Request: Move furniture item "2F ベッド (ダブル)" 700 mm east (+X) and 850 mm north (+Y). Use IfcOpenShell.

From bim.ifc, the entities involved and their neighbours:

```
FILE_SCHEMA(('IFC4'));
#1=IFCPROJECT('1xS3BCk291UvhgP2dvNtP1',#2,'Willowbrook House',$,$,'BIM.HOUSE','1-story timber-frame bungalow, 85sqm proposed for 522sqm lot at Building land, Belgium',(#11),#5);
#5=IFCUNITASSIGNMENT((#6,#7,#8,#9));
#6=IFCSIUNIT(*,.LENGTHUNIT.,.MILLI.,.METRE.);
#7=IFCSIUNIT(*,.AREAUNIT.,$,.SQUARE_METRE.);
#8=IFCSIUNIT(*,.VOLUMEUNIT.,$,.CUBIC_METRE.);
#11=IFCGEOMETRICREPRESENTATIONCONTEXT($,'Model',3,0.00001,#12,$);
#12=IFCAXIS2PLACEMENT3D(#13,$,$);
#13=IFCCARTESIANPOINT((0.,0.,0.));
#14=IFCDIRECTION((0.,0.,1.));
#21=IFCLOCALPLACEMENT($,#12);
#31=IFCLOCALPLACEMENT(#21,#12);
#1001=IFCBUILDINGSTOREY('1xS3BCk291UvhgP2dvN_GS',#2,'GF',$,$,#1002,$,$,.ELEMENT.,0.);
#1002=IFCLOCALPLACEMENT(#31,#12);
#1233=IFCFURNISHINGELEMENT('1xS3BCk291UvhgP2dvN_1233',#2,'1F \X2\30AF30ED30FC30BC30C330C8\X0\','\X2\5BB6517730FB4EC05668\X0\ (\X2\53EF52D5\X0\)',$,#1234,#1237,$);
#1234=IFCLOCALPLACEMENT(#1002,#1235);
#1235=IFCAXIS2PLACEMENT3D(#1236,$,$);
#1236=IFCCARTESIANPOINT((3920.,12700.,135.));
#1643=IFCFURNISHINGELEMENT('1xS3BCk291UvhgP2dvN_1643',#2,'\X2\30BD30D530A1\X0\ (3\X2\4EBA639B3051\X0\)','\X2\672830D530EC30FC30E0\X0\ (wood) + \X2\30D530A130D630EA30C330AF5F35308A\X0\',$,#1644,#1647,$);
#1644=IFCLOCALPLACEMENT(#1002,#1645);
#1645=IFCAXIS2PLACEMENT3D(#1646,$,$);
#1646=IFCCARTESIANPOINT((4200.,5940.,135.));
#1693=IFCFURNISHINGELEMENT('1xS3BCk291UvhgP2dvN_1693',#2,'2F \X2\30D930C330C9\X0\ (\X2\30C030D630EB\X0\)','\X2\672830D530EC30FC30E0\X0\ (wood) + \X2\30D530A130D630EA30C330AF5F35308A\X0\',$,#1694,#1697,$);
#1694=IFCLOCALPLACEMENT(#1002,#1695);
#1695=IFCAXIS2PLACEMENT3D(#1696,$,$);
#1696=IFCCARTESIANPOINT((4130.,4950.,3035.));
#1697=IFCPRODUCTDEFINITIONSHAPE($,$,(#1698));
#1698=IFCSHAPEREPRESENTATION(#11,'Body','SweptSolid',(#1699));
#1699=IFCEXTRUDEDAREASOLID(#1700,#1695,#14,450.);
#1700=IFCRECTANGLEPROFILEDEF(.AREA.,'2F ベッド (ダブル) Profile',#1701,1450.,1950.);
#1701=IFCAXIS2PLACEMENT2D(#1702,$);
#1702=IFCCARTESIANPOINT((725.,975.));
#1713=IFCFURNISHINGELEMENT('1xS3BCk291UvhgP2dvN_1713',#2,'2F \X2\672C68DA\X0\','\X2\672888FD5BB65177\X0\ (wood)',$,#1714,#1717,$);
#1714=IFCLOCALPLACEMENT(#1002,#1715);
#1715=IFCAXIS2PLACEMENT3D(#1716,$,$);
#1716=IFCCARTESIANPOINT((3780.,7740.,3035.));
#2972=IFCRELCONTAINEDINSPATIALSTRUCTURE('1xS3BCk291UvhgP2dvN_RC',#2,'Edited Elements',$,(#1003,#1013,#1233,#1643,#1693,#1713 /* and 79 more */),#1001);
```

```python
import ifcopenshell
import ifcopenshell.api.geometry
import ifcopenshell.util.placement
import ifcopenshell.util.unit

model = ifcopenshell.open("bim.ifc")
unit_scale = ifcopenshell.util.unit.calculate_unit_scale(model)

item = model.by_guid("1xS3BCk291UvhgP2dvN_1693")
matrix = ifcopenshell.util.placement.get_local_placement(item.ObjectPlacement)
matrix[0, 3] += 0.7 / unit_scale
matrix[1, 3] += 0.85 / unit_scale
ifcopenshell.api.geometry.edit_object_placement(model, product=item, matrix=matrix, is_si=False)

print(ifcopenshell.util.placement.get_local_placement(item.ObjectPlacement).round(3) + 0.0)

model.write("bim_v2.ifc")
```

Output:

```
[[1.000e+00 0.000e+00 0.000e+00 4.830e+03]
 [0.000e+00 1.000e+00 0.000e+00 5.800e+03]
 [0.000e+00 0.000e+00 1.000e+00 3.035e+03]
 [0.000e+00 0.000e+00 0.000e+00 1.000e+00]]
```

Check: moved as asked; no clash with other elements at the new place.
